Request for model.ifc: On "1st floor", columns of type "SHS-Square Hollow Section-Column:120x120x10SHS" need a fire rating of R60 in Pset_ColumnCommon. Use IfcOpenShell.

First a look at what the model holds.

```python
import ifcopenshell
import ifcopenshell.util.element

model = ifcopenshell.open("model.ifc")
print(model.schema)
storey = next(s for s in model.by_type("IfcBuildingStorey") if s.Name == "1st floor")
columns = [e for e in ifcopenshell.util.element.get_decomposition(storey) if e.is_a("IfcColumn")]
seen = {}
for e in columns:
    element_type = ifcopenshell.util.element.get_type(e)
    key = (element_type.Name if element_type != e and element_type else None, ifcopenshell.util.element.get_pset(e, "Pset_ColumnCommon", "FireRating"))
    seen[key] = seen.get(key, 0) + 1
for (name, value), count in sorted(seen.items(), key=str):
    print(count, "x", name, "|", value)
```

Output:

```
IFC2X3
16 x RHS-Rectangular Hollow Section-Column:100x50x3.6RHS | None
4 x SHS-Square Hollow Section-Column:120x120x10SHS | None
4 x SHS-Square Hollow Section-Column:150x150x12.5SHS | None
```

```python
import ifcopenshell
import ifcopenshell.api.pset
import ifcopenshell.util.element

model = ifcopenshell.open("model.ifc")

storey = next(s for s in model.by_type("IfcBuildingStorey") if s.Name == "1st floor")
columns = [e for e in ifcopenshell.util.element.get_decomposition(storey) if e.is_a("IfcColumn")]

count = 0
for e in columns:
    element_type = ifcopenshell.util.element.get_type(e)
    if element_type in (None, e) or element_type.Name != "SHS-Square Hollow Section-Column:120x120x10SHS":
        continue
    # add_pset returns the element's existing set when there is one.
    pset = ifcopenshell.api.pset.add_pset(model, product=e, name="Pset_ColumnCommon")
    ifcopenshell.api.pset.edit_pset(model, pset=pset, properties={"FireRating": "R60"})
    count += 1

print(count, "columns updated")

model.write("model-out.ifc")
```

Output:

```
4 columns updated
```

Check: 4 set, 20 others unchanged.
